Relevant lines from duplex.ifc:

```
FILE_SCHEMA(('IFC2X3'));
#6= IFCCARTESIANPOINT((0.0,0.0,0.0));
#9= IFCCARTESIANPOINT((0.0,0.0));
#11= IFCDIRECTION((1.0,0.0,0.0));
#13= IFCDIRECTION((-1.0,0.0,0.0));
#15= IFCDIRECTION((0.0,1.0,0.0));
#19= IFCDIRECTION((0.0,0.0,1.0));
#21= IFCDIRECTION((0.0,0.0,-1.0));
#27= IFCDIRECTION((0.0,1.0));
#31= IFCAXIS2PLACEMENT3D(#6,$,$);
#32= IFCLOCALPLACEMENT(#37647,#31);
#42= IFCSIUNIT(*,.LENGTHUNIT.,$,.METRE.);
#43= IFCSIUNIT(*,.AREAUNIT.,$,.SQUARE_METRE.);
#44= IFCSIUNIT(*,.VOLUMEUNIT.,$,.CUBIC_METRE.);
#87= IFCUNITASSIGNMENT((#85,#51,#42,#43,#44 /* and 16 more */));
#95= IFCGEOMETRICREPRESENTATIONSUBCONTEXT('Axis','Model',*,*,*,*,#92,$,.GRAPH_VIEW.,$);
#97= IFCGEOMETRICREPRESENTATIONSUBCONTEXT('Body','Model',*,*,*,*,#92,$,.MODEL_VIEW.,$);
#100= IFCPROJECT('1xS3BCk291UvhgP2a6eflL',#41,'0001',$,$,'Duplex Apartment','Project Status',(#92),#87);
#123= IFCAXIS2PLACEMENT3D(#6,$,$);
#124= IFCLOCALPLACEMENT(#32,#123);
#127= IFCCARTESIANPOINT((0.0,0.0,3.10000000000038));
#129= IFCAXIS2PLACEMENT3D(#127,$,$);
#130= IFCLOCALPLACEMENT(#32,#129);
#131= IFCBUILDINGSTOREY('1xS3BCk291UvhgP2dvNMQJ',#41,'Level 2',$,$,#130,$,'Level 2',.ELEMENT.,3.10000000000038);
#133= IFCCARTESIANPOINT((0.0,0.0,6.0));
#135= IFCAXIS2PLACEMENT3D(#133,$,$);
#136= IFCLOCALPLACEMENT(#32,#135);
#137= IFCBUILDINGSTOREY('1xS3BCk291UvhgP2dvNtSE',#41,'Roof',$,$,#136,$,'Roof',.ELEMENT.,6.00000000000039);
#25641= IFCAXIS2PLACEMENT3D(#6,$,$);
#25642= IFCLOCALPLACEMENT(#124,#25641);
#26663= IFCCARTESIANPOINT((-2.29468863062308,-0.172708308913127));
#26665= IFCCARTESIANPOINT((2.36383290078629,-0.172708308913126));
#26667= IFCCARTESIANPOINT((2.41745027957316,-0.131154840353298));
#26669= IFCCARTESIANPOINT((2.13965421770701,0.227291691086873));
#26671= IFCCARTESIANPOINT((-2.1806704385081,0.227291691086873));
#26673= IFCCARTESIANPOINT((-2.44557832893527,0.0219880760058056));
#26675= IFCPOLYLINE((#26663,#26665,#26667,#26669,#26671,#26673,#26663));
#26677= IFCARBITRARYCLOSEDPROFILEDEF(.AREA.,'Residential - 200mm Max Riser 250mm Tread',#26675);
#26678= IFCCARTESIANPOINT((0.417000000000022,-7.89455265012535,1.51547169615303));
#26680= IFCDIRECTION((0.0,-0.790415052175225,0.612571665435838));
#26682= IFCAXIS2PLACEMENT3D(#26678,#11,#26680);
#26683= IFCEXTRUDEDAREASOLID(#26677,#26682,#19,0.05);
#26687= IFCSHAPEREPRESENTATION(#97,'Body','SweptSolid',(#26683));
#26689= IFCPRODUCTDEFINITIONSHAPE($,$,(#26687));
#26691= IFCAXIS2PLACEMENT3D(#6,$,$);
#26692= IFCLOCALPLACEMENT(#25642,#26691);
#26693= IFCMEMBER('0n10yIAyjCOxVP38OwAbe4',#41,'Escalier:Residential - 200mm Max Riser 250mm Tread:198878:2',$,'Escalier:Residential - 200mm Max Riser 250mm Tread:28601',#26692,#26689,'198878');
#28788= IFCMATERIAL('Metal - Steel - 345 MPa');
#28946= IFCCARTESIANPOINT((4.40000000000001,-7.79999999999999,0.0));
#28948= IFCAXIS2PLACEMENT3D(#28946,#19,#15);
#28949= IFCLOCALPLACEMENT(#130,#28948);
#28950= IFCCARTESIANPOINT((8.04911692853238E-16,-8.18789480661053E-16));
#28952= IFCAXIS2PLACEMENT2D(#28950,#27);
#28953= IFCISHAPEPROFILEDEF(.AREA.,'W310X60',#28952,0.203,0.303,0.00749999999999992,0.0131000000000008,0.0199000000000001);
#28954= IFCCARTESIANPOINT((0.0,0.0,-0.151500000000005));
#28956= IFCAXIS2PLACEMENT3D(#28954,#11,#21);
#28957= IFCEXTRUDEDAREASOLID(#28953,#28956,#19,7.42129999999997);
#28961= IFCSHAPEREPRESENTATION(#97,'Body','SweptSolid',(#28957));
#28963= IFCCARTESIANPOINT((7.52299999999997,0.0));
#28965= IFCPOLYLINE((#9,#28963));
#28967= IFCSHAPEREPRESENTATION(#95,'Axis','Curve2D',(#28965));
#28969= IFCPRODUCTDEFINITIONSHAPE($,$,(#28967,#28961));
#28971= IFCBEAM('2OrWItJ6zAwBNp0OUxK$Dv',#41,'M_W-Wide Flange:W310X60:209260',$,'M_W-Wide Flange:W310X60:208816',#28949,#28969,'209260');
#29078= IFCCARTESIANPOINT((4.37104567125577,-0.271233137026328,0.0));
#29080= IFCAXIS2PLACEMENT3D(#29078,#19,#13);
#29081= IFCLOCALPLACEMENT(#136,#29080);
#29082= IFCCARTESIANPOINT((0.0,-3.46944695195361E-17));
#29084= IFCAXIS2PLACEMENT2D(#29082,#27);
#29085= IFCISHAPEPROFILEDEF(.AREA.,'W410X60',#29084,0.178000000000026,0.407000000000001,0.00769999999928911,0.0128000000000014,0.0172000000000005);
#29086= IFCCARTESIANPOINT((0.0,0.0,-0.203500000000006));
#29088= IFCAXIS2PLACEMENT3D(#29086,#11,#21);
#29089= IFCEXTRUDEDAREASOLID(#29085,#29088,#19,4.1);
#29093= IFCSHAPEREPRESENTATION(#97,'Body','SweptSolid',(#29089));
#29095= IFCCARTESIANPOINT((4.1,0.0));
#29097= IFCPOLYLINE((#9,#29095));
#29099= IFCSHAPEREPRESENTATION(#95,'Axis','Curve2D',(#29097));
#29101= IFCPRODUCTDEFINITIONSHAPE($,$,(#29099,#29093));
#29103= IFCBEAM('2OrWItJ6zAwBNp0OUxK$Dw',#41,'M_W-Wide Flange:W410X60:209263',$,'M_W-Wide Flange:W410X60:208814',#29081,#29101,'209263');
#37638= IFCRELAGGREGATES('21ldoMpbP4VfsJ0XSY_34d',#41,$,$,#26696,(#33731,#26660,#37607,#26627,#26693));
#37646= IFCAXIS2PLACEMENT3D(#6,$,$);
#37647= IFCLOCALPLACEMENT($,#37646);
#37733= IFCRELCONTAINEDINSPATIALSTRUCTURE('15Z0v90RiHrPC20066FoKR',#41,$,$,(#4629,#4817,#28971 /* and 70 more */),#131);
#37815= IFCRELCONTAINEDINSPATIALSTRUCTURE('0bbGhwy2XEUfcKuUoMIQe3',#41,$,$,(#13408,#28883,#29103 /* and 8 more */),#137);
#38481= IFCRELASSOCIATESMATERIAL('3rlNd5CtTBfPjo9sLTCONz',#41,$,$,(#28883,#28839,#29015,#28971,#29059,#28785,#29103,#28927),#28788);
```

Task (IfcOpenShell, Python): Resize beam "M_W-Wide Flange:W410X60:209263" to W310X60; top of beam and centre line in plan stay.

```python
import ifcopenshell
import ifcopenshell.util.element
import ifcopenshell.util.representation

model = ifcopenshell.open("duplex.ifc")

member = model.by_guid("2OrWItJ6zAwBNp0OUxK$Dw")
source = next(p for p in model.by_type("IfcIShapeProfileDef") if p.ProfileName == "W310X60")

body = ifcopenshell.util.representation.get_representation(member, "Model", "Body")
solid = body.Items[0]
old_profile = solid.SweptArea

# Copy the section's sizes but keep this member's own profile position.
profile = ifcopenshell.util.element.copy(model, source)
# Profiles are centred, so shift by half the change in depth to hold the top.
shift = (old_profile.OverallDepth - profile.OverallDepth) / 2
x, y = old_profile.Position.Location.Coordinates
up = (-1.0, 0.0)  # upwards, in the solid's own plane
location = model.createIfcCartesianPoint((x + up[0] * shift, y + up[1] * shift))
profile.Position = model.createIfcAxis2Placement2D(location, old_profile.Position.RefDirection)
solid.SweptArea = profile
if not model.get_total_inverses(old_profile):
    ifcopenshell.util.element.remove_deep2(model, old_profile)
member.Name = member.Name.replace("W410X60", "W310X60")
member.ObjectType = member.ObjectType.replace("W410X60", "W310X60")

print(solid.SweptArea)

model.write("duplex-out.ifc")
```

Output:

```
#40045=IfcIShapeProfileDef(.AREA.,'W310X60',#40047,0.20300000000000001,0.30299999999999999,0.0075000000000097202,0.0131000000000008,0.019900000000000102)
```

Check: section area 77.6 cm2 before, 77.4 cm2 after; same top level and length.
